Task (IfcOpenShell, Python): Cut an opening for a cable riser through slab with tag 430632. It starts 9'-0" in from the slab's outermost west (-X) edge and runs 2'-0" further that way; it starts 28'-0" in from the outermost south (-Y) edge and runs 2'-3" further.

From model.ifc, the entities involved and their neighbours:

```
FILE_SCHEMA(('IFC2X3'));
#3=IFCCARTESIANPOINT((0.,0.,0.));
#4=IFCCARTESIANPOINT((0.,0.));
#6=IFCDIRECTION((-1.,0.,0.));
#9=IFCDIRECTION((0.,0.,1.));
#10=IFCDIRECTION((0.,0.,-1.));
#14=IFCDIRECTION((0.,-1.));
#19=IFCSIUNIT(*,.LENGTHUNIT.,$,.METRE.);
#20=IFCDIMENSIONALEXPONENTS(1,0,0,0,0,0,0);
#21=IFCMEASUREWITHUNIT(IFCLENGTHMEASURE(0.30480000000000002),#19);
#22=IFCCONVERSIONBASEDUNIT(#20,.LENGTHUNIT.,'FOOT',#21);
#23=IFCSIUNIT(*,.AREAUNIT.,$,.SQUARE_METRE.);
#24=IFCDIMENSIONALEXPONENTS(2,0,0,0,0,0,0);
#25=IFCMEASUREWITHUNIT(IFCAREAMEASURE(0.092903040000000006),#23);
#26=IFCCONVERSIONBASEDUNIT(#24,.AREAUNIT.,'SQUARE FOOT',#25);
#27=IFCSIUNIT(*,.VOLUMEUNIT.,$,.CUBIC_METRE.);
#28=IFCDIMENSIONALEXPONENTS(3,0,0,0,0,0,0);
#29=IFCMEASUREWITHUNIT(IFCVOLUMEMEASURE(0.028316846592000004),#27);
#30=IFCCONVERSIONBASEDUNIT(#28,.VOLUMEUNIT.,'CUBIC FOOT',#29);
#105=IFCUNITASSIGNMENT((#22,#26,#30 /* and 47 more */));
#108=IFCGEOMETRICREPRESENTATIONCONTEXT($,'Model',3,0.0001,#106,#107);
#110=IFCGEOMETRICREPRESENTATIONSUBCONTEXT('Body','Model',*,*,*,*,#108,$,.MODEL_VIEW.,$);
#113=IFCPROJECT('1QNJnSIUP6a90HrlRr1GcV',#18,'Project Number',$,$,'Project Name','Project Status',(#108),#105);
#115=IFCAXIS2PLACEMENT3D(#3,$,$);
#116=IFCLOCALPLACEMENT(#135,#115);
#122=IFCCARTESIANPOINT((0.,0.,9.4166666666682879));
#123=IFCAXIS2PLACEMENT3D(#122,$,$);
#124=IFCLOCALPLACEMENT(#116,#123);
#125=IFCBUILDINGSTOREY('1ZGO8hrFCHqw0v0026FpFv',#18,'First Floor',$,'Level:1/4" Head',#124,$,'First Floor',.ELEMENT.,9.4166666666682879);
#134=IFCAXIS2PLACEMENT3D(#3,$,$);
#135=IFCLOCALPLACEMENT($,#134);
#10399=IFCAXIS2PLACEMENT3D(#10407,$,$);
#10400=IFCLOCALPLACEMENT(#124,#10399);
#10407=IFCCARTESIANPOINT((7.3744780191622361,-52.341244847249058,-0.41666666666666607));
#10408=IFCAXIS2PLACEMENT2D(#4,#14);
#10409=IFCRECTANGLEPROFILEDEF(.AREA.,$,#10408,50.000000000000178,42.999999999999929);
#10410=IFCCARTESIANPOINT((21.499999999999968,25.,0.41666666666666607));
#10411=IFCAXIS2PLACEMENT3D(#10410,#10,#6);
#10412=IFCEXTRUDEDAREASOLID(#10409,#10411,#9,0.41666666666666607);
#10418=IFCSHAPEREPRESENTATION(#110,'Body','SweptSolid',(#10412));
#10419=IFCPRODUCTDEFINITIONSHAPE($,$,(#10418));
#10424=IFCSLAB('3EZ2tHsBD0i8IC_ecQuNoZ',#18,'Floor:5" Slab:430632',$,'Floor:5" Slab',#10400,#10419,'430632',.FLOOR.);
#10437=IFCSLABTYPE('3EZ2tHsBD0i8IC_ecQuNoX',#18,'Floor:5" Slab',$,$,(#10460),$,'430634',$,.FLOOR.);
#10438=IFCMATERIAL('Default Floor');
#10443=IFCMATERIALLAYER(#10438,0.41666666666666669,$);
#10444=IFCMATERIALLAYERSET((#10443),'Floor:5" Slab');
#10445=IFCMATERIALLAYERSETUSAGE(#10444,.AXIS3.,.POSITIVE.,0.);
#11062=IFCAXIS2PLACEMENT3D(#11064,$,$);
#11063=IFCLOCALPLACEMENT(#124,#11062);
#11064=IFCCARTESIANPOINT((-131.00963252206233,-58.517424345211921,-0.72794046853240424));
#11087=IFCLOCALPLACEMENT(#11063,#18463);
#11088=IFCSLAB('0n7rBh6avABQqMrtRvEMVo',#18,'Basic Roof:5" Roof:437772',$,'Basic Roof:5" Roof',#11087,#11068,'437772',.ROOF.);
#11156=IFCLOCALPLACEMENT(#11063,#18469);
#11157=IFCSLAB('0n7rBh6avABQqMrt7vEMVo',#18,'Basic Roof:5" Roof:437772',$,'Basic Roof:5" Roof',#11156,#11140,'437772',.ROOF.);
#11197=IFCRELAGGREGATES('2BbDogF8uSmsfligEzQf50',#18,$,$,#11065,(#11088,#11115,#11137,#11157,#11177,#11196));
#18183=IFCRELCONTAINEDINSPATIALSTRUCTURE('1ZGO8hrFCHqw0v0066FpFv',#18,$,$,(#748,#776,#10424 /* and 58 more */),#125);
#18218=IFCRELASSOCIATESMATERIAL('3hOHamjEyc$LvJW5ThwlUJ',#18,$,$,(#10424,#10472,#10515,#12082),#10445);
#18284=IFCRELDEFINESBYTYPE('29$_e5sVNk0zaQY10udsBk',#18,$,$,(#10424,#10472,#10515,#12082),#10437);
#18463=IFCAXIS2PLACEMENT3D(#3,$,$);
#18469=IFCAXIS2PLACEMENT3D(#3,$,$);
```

```python
import numpy as np
import ifcopenshell
import ifcopenshell.api.feature
import ifcopenshell.api.geometry
import ifcopenshell.api.root
import ifcopenshell.geom
import ifcopenshell.util.placement
import ifcopenshell.util.representation
import ifcopenshell.util.shape
import ifcopenshell.util.unit

model = ifcopenshell.open("model.ifc")
unit_scale = ifcopenshell.util.unit.calculate_unit_scale(model)
settings = ifcopenshell.geom.settings()


def volume(element):
    """Net volume in cubic metres, openings subtracted."""
    shape = ifcopenshell.geom.create_shape(settings, element)
    return ifcopenshell.util.shape.get_volume(shape.geometry)


slab = model.by_id(10424)
before = volume(slab)

# Extent in the slab's own axes, in metres. The edges named are its -X and -Y sides.
slab_shape = ifcopenshell.geom.create_shape(settings, slab)
vertices = ifcopenshell.util.shape.get_vertices(slab_shape.geometry)
x_min, y_min, bottom = vertices.min(axis=0)
top = vertices[:, 2].max()

opening = ifcopenshell.api.root.create_entity(model, ifc_class="IfcOpeningElement", name="Cable riser opening")
context = ifcopenshell.util.representation.get_context(model, "Model", "Body", "MODEL_VIEW")
width, depth = 0.6096, 0.6858
outline = [(0.0, 0.0), (width, 0.0), (width, depth), (0.0, depth), (0.0, 0.0)]
# Overshoot both faces by 50 mm so the cut is clean.
shape = ifcopenshell.api.geometry.add_slab_representation(
    model, context=context, depth=top - bottom + 0.1, polyline=outline
)
ifcopenshell.api.geometry.assign_representation(model, product=opening, representation=shape)

matrix = ifcopenshell.util.placement.get_local_placement(slab.ObjectPlacement)
matrix[:, 3] = matrix @ np.append(np.array([x_min + 2.7432, y_min + 8.5344, bottom - 0.05]) / unit_scale, 1.0)
ifcopenshell.api.geometry.edit_object_placement(model, product=opening, matrix=matrix, is_si=False)
ifcopenshell.api.feature.add_feature(model, feature=opening, element=slab)

after = volume(slab)

print(f"slab volume {before:.3f} -> {after:.3f} m3")

model.write("model_updated.ifc")
```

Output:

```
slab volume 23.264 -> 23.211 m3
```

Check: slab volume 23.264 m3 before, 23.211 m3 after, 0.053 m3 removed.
